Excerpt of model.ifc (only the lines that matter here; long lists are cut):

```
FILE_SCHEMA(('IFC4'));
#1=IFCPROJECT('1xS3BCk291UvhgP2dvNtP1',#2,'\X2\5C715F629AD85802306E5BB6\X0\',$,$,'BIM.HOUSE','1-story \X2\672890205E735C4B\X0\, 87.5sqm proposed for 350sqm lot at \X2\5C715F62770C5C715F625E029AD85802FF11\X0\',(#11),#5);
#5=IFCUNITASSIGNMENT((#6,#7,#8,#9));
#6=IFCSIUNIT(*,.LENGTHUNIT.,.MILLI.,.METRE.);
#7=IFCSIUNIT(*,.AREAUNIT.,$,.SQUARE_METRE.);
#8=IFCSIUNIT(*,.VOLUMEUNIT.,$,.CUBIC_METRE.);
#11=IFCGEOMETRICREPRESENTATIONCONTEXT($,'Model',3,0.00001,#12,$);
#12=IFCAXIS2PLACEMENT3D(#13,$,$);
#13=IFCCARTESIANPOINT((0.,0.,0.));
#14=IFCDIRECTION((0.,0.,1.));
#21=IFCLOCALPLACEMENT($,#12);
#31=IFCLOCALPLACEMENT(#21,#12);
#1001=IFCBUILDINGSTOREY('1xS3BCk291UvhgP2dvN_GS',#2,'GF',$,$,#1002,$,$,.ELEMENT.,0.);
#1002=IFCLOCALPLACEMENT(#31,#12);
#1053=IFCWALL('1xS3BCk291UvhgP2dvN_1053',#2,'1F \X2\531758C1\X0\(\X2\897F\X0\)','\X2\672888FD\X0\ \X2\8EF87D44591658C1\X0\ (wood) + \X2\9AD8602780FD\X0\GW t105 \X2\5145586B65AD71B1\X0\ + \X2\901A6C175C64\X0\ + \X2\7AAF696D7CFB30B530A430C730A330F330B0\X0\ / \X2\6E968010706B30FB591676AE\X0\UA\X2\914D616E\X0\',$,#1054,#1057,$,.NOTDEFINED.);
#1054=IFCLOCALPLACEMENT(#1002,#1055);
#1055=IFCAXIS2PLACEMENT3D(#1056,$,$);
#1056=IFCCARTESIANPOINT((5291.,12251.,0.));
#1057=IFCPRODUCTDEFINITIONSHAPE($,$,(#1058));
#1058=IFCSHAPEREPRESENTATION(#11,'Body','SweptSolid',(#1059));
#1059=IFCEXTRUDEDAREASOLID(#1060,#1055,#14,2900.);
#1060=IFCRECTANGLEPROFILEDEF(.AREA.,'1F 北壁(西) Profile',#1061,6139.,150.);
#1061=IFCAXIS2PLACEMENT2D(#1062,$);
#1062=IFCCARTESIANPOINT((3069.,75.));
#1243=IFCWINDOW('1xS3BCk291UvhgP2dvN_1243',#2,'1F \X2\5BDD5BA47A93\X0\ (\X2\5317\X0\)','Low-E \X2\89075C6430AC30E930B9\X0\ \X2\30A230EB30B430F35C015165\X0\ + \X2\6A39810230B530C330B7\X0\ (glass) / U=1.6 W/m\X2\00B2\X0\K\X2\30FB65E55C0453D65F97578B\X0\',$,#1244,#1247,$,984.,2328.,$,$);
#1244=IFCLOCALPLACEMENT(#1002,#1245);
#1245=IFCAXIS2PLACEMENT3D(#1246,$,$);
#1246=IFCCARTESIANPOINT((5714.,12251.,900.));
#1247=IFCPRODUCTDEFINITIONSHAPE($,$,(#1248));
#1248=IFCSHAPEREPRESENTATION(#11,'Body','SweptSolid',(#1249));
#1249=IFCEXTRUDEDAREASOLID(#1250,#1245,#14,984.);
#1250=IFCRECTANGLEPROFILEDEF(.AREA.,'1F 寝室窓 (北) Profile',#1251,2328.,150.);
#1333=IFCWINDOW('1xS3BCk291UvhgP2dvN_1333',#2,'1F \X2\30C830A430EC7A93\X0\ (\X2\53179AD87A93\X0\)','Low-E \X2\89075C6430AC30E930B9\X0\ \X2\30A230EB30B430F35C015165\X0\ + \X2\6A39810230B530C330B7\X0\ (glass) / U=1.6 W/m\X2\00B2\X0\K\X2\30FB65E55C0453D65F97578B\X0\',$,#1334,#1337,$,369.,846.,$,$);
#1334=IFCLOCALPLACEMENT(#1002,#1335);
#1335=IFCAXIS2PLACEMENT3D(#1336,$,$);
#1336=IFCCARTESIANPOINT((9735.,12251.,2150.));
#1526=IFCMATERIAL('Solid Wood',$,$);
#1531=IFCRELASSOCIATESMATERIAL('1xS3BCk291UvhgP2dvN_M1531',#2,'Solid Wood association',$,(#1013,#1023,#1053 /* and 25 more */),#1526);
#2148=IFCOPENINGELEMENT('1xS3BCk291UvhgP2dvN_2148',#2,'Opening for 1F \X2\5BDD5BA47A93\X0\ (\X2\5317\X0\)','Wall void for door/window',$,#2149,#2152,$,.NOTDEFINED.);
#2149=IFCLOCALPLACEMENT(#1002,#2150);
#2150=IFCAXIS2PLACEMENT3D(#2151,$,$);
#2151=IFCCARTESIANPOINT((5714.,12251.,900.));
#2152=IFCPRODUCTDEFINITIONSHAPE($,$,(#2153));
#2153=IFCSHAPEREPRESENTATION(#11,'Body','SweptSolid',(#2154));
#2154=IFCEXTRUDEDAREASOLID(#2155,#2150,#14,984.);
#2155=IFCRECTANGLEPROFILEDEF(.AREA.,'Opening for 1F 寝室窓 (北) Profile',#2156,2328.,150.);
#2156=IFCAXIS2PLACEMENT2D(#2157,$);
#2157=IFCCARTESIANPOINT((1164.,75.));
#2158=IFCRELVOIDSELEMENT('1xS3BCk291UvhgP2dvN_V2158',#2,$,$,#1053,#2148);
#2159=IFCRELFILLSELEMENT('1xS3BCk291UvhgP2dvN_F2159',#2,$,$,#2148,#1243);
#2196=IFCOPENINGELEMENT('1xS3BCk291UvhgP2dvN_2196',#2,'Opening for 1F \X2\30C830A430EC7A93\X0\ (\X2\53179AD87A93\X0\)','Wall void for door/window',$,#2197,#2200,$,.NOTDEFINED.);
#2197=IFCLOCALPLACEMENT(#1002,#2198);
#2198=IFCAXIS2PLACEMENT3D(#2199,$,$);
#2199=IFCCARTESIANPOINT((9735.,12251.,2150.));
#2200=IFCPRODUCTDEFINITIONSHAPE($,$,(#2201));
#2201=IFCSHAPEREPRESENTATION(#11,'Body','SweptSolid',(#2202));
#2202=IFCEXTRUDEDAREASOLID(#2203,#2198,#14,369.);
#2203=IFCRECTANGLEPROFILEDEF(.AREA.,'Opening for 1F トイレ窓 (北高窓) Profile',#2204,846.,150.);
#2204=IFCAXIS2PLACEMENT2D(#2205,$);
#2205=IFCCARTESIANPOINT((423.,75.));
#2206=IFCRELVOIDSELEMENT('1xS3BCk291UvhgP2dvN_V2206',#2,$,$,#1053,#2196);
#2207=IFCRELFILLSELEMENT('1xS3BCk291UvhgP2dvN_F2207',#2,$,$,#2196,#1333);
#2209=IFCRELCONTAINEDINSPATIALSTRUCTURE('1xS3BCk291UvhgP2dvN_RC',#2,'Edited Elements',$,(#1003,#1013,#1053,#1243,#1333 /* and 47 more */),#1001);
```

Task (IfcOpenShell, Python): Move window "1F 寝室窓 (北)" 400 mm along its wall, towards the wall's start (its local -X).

```python
import ifcopenshell
import ifcopenshell.api.geometry
import ifcopenshell.util.placement
import ifcopenshell.util.unit

model = ifcopenshell.open("model.ifc")
unit_scale = ifcopenshell.util.unit.calculate_unit_scale(model)

window = model.by_id(1243)
opening = window.FillsVoids[0].RelatingOpeningElement
wall = opening.VoidsElements[0].RelatingBuildingElement

wall_matrix = ifcopenshell.util.placement.get_local_placement(wall.ObjectPlacement)
shift = wall_matrix[:3, 0] * -0.4 / unit_scale
before = ifcopenshell.util.placement.get_local_placement(window.ObjectPlacement)[:3, 3].copy()

# The window is not placed relative to its opening, so move both.
for product in (opening, window):
    matrix = ifcopenshell.util.placement.get_local_placement(product.ObjectPlacement)
    matrix[:3, 3] += shift
    ifcopenshell.api.geometry.edit_object_placement(model, product=product, matrix=matrix, is_si=False)

after = ifcopenshell.util.placement.get_local_placement(window.ObjectPlacement)[:3, 3]
print("window moved by", (after - before).round(3) + 0.0)

model.write("model_v2.ifc")
```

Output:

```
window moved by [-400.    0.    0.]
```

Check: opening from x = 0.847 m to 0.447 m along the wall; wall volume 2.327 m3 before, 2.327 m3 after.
